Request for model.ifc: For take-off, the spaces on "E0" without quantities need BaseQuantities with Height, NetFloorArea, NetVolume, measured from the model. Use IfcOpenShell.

First a look at what the model holds.

```python
import ifcopenshell
import ifcopenshell.util.element
import ifcopenshell.util.unit

model = ifcopenshell.open("model.ifc")
print(model.schema)
for unit_type in ("LENGTHUNIT", "AREAUNIT", "VOLUMEUNIT"):
    print(unit_type, ifcopenshell.util.unit.calculate_unit_scale(model, unit_type))
storey = next(s for s in model.by_type("IfcBuildingStorey") if s.Name == "E0")
spaces = [e for e in ifcopenshell.util.element.get_decomposition(storey) if e.is_a("IfcSpace")]
for e in sorted(spaces, key=lambda e: e.id()):
    print(e.id(), e.is_a(), e.Name, list(ifcopenshell.util.element.get_psets(e, qtos_only=True)), sep=" | ")
```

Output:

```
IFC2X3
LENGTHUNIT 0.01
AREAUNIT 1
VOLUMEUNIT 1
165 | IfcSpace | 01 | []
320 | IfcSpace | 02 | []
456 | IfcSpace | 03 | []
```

```python
import ifcopenshell
import ifcopenshell.api.pset
import ifcopenshell.geom
import ifcopenshell.util.element
import ifcopenshell.util.shape
import ifcopenshell.util.unit

model = ifcopenshell.open("model.ifc")
unit_scale = ifcopenshell.util.unit.calculate_unit_scale(model)
area_scale = ifcopenshell.util.unit.calculate_unit_scale(model, "AREAUNIT")
volume_scale = ifcopenshell.util.unit.calculate_unit_scale(model, "VOLUMEUNIT")
settings = ifcopenshell.geom.settings()

storey = next(s for s in model.by_type("IfcBuildingStorey") if s.Name == "E0")
spaces = [e for e in ifcopenshell.util.element.get_decomposition(storey) if e.is_a("IfcSpace")]

for e in sorted(spaces, key=lambda e: e.id()):
    if ifcopenshell.util.element.get_psets(e, qtos_only=True, should_inherit=False):
        continue
    # Geometry comes back in metres, in the element's own axes.
    shape = ifcopenshell.geom.create_shape(settings, e)
    values = {
        "Height": ifcopenshell.util.shape.get_z(shape.geometry) / unit_scale,
        "NetFloorArea": ifcopenshell.util.shape.get_footprint_area(shape.geometry) / area_scale,
        "NetVolume": ifcopenshell.util.shape.get_volume(shape.geometry) / volume_scale,
    }
    qto = ifcopenshell.api.pset.add_qto(model, product=e, name="BaseQuantities")
    ifcopenshell.api.pset.edit_qto(model, qto=qto, properties=values)
    print(e.id(), {k: round(v, 3) for k, v in values.items()})

model.write("model_v2.ifc")
```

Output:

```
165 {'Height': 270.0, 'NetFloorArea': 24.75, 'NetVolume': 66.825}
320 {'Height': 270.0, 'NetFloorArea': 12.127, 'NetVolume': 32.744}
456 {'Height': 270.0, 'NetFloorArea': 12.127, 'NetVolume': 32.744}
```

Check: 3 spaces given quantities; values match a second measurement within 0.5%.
